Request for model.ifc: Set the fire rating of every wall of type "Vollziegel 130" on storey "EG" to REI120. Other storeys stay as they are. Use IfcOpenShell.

First a look at what the model holds.

```python
import ifcopenshell
import ifcopenshell.util.element

model = ifcopenshell.open("model.ifc")
print(model.schema)
storey = next(s for s in model.by_type("IfcBuildingStorey") if s.Name == "EG")
walls = [e for e in ifcopenshell.util.element.get_decomposition(storey) if e.is_a("IfcWall")]
seen = {}
for e in walls:
    element_type = ifcopenshell.util.element.get_type(e)
    key = (element_type.Name if element_type != e and element_type else None, ifcopenshell.util.element.get_pset(e, "Pset_WallCommon", "FireRating"))
    seen[key] = seen.get(key, 0) + 1
for (name, value), count in sorted(seen.items(), key=str):
    print(count, "x", name, "|", value)
```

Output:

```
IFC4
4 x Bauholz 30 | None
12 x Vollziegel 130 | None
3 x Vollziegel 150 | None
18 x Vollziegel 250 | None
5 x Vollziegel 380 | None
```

```python
import ifcopenshell
import ifcopenshell.api.pset
import ifcopenshell.util.element

model = ifcopenshell.open("model.ifc")

storey = next(s for s in model.by_type("IfcBuildingStorey") if s.Name == "EG")
walls = [e for e in ifcopenshell.util.element.get_decomposition(storey) if e.is_a("IfcWall")]

count = 0
for e in walls:
    element_type = ifcopenshell.util.element.get_type(e)
    if element_type in (None, e) or element_type.Name != "Vollziegel 130":
        continue
    # add_pset returns the element's existing set when there is one.
    pset = ifcopenshell.api.pset.add_pset(model, product=e, name="Pset_WallCommon")
    ifcopenshell.api.pset.edit_pset(model, pset=pset, properties={"FireRating": "REI120"})
    count += 1

print(count, "walls updated")

model.write("model_v2.ifc")
```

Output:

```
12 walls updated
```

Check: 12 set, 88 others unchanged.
